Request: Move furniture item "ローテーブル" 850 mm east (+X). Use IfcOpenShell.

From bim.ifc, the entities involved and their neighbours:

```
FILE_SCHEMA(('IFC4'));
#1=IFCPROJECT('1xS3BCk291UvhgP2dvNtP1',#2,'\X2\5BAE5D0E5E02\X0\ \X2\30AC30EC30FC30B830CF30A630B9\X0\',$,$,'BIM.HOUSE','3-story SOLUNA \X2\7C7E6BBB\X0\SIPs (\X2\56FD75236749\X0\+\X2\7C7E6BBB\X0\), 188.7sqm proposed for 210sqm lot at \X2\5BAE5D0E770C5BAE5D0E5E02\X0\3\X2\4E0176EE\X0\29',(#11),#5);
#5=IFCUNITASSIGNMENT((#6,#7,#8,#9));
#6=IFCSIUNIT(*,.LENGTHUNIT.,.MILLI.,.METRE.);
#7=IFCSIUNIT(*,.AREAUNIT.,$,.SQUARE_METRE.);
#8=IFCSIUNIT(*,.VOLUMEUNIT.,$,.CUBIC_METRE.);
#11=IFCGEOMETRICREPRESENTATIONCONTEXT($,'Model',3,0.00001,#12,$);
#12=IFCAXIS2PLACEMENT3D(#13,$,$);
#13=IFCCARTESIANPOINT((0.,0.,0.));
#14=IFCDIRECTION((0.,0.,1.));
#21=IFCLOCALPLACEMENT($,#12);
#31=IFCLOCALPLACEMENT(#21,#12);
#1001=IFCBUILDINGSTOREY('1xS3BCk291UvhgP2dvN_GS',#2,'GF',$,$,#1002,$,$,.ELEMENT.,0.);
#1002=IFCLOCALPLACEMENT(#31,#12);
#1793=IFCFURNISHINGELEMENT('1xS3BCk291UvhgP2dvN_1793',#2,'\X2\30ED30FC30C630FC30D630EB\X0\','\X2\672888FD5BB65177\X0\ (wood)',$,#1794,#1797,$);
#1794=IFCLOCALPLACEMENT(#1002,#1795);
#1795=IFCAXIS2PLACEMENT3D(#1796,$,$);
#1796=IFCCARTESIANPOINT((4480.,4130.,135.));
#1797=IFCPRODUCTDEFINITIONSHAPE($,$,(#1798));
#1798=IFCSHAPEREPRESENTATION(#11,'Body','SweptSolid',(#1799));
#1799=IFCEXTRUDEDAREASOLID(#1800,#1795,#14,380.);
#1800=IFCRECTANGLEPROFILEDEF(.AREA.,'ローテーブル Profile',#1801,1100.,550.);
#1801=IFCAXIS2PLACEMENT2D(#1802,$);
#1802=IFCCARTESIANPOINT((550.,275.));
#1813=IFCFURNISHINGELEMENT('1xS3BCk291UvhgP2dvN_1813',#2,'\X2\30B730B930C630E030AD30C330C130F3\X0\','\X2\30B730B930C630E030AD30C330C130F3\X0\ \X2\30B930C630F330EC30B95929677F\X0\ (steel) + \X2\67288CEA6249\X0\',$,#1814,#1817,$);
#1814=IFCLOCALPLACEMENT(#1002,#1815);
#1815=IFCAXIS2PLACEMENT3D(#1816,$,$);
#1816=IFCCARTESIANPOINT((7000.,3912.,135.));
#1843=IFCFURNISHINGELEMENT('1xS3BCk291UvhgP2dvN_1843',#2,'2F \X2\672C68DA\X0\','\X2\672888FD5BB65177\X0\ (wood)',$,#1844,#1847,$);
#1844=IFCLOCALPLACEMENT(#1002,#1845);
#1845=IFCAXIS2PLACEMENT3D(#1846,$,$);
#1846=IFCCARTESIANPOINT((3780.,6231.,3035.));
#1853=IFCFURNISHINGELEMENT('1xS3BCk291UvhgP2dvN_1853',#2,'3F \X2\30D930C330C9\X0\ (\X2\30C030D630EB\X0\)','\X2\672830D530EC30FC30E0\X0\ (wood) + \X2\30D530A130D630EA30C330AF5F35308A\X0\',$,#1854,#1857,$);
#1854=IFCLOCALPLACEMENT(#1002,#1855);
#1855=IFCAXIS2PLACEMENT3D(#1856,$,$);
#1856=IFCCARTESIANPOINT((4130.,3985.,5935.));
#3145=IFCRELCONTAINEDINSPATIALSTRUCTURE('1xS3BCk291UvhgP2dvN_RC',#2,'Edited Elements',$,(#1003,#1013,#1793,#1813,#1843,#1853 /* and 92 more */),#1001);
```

```python
import ifcopenshell
import ifcopenshell.api.geometry
import ifcopenshell.util.placement

model = ifcopenshell.open("bim.ifc")

item = model.by_guid("1xS3BCk291UvhgP2dvN_1793")
matrix = ifcopenshell.util.placement.get_local_placement(item.ObjectPlacement)
matrix[0, 3] += 850.0
ifcopenshell.api.geometry.edit_object_placement(model, product=item, matrix=matrix, is_si=False)

print(ifcopenshell.util.placement.get_local_placement(item.ObjectPlacement).round(3) + 0.0)

model.write("bim_edited.ifc")
```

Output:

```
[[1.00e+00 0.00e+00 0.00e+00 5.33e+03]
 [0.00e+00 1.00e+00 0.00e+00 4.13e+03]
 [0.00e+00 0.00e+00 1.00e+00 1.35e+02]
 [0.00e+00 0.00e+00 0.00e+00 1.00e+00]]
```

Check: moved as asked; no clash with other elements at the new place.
